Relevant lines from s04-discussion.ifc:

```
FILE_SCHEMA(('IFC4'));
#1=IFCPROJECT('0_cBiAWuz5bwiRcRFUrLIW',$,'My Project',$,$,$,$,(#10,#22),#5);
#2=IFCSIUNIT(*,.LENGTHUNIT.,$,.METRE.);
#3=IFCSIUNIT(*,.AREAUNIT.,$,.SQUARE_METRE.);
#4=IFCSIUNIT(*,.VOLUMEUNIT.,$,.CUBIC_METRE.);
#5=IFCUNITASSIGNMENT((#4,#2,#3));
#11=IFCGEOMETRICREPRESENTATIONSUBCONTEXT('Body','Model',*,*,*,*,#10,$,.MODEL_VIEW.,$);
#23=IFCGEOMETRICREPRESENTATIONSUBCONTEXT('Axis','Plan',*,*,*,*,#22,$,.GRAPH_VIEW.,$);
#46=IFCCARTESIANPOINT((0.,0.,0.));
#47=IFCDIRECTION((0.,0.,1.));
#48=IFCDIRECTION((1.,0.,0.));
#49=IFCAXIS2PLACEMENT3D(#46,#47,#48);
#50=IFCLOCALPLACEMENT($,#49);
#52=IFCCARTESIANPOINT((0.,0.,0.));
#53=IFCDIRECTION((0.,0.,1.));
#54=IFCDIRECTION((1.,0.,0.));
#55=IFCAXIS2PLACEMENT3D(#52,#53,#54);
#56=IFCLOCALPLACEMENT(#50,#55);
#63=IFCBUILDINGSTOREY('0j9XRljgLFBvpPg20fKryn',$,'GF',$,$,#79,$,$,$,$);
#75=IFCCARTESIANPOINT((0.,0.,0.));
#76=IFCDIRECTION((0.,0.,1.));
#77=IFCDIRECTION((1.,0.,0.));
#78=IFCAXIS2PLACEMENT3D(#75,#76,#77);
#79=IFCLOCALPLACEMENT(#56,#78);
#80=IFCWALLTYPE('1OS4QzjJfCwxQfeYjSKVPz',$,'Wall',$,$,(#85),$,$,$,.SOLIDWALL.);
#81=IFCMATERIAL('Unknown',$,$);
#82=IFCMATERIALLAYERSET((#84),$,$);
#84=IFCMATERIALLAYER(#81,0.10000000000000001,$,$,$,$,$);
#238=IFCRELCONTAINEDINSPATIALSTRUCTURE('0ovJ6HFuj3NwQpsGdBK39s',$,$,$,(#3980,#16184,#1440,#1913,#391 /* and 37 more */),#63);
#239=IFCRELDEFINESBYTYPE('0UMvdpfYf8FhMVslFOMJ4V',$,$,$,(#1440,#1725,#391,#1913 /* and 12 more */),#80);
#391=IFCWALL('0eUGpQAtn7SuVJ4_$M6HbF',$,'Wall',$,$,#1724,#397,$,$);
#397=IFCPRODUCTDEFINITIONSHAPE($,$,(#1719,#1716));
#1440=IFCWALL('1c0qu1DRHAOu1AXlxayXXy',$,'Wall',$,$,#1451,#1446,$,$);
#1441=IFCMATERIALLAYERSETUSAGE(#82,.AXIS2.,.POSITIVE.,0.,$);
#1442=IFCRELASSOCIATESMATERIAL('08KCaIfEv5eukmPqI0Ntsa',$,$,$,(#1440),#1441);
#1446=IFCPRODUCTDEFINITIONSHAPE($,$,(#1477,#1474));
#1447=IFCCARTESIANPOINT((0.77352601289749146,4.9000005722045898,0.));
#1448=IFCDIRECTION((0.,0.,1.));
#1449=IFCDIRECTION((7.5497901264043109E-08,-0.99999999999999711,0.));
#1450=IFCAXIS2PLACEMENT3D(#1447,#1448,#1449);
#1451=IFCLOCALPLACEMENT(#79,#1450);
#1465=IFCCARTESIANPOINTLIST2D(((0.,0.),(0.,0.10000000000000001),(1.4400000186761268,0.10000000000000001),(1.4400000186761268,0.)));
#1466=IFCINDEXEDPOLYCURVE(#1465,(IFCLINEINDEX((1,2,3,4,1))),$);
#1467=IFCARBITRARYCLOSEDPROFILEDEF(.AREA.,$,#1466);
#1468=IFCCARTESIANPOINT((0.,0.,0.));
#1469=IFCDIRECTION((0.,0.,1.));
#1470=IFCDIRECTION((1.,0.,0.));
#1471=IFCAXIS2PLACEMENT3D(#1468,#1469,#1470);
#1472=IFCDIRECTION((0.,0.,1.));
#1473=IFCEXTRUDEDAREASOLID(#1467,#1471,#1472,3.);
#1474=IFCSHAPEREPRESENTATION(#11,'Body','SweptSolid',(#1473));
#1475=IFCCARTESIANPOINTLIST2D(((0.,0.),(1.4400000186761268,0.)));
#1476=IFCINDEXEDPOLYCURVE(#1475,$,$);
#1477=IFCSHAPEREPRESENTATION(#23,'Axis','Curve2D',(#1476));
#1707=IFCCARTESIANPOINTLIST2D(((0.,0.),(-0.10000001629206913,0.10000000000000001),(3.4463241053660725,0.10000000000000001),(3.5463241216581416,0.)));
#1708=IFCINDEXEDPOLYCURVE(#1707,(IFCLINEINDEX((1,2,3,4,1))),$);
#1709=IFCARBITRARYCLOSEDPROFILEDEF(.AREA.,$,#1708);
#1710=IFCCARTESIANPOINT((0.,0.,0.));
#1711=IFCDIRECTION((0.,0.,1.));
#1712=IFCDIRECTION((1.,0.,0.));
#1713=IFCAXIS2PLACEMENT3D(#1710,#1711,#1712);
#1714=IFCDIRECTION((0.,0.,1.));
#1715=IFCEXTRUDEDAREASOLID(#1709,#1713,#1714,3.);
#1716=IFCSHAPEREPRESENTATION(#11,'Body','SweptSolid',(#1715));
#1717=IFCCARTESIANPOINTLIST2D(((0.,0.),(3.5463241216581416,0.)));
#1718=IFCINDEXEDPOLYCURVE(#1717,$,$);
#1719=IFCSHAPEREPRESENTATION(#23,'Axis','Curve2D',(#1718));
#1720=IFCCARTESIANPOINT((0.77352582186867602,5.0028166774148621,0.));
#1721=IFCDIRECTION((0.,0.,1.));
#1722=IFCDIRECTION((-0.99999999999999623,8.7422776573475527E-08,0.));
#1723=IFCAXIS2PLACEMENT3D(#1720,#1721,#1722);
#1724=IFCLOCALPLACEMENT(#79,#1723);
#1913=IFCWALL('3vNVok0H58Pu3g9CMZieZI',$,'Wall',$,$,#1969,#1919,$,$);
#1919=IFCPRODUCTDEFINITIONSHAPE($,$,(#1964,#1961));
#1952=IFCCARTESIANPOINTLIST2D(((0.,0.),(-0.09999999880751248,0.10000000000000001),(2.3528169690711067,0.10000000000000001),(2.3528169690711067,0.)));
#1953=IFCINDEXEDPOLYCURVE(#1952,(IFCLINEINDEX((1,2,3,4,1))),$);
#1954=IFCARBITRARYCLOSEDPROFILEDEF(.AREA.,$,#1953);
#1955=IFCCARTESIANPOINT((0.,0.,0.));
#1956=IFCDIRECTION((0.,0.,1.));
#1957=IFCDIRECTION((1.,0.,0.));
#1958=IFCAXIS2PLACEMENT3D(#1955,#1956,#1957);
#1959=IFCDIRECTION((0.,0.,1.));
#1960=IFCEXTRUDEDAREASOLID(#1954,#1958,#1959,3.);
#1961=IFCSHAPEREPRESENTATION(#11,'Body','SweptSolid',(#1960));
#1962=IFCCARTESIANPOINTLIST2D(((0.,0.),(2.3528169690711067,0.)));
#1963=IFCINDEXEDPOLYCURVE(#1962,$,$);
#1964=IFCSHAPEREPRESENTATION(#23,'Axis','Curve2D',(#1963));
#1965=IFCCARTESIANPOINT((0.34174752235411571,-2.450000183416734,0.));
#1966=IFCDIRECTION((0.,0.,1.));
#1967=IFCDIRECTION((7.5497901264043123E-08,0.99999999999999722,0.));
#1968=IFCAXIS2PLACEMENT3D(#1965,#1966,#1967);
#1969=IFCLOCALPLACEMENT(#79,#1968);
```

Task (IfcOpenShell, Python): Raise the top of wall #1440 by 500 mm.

```python
import ifcopenshell
import ifcopenshell.geom
import ifcopenshell.util.representation
import ifcopenshell.util.shape
import ifcopenshell.util.unit

model = ifcopenshell.open("s04-discussion.ifc")
unit_scale = ifcopenshell.util.unit.calculate_unit_scale(model)
settings = ifcopenshell.geom.settings()


def volume(element):
    """Net volume in cubic metres, openings subtracted."""
    shape = ifcopenshell.geom.create_shape(settings, element)
    return ifcopenshell.util.shape.get_volume(shape.geometry)


wall = model.by_guid("1c0qu1DRHAOu1AXlxayXXy")
before = volume(wall)

body = ifcopenshell.util.representation.get_representation(wall, "Model", "Body")
solid = body.Items[0]
old_height = solid.Depth
solid.Depth += 0.5 / unit_scale
after = volume(wall)

print(f"height {old_height:g} -> {solid.Depth:g}, volume {before:.3f} -> {after:.3f} m3")

model.write("s04-discussion-out.ifc")
```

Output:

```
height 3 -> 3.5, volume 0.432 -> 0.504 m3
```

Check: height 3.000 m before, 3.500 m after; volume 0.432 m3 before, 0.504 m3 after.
